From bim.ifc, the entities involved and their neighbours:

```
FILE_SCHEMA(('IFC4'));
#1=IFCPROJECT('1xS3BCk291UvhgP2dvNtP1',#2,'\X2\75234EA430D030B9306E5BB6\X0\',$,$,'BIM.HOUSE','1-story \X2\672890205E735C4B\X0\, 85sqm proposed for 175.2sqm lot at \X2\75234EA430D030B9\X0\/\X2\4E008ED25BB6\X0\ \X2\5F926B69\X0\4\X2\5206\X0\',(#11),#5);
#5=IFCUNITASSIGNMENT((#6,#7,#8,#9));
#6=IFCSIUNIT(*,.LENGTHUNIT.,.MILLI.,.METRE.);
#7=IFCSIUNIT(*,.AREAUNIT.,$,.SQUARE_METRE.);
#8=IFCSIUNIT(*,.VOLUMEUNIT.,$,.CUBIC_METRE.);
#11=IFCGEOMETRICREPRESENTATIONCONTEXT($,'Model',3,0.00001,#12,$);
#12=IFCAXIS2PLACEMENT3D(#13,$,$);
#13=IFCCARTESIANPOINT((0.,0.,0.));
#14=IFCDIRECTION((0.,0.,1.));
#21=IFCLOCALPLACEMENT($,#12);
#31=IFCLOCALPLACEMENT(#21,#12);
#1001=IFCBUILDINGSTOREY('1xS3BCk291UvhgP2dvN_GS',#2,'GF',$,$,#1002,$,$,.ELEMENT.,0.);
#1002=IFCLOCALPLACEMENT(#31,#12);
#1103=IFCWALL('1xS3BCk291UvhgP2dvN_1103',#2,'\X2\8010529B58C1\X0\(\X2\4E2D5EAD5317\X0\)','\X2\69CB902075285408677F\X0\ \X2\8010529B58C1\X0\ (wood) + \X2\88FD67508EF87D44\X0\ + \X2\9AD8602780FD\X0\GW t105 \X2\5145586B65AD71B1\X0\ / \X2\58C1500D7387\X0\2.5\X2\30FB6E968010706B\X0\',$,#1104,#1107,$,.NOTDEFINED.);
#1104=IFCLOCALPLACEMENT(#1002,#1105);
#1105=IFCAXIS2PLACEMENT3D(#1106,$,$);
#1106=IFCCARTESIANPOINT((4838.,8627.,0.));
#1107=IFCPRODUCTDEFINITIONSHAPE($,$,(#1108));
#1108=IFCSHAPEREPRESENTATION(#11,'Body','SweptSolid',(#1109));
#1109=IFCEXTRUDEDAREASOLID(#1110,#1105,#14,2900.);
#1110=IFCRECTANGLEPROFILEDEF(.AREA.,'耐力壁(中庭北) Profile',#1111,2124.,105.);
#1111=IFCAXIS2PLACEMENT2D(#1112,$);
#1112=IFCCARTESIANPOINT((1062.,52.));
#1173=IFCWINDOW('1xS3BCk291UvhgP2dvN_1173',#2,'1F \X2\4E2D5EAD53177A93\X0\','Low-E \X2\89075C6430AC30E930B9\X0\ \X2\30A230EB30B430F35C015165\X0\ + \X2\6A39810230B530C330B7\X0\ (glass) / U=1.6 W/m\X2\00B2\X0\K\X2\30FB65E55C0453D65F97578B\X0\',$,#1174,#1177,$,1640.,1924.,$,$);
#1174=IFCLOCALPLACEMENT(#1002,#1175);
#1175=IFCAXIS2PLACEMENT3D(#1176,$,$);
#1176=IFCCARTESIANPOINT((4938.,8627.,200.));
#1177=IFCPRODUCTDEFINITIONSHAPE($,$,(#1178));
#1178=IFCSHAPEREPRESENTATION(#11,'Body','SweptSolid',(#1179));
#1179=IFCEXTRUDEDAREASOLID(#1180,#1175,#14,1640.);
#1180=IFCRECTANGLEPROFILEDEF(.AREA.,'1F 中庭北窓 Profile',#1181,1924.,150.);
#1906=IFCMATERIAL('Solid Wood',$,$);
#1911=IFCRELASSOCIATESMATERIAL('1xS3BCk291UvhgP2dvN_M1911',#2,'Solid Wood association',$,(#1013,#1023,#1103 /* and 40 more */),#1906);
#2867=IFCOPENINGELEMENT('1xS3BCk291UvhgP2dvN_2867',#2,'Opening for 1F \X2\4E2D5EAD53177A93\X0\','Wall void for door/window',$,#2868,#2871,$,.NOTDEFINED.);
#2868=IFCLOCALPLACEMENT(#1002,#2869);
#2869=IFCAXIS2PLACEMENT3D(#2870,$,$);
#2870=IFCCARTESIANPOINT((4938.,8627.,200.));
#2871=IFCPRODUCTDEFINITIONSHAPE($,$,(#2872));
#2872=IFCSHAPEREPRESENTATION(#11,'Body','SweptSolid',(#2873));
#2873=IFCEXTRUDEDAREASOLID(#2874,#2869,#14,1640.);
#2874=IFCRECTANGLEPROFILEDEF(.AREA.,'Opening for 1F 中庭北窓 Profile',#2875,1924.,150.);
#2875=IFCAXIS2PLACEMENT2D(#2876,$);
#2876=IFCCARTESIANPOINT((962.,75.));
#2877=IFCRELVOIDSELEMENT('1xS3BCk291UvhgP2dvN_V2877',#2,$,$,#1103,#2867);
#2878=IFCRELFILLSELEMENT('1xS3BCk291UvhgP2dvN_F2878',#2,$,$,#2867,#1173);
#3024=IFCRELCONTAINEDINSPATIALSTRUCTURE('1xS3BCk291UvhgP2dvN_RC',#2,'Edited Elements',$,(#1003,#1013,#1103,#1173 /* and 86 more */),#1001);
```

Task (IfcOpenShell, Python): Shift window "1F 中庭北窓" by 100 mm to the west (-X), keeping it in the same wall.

```python
import ifcopenshell
import ifcopenshell.api.geometry
import ifcopenshell.util.placement

model = ifcopenshell.open("bim.ifc")

window = model.by_id(1173)
opening = window.FillsVoids[0].RelatingOpeningElement
wall = opening.VoidsElements[0].RelatingBuildingElement

wall_matrix = ifcopenshell.util.placement.get_local_placement(wall.ObjectPlacement)
shift = wall_matrix[:3, 0] * -100.0
before = ifcopenshell.util.placement.get_local_placement(window.ObjectPlacement)[:3, 3].copy()

# The window is not placed relative to its opening, so move both.
for product in (opening, window):
    matrix = ifcopenshell.util.placement.get_local_placement(product.ObjectPlacement)
    matrix[:3, 3] += shift
    ifcopenshell.api.geometry.edit_object_placement(model, product=product, matrix=matrix, is_si=False)

after = ifcopenshell.util.placement.get_local_placement(window.ObjectPlacement)[:3, 3]
print("window moved by", (after - before).round(3) + 0.0)

model.write("bim-out.ifc")
```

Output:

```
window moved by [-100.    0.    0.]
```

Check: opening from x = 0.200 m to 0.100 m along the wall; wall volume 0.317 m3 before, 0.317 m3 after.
